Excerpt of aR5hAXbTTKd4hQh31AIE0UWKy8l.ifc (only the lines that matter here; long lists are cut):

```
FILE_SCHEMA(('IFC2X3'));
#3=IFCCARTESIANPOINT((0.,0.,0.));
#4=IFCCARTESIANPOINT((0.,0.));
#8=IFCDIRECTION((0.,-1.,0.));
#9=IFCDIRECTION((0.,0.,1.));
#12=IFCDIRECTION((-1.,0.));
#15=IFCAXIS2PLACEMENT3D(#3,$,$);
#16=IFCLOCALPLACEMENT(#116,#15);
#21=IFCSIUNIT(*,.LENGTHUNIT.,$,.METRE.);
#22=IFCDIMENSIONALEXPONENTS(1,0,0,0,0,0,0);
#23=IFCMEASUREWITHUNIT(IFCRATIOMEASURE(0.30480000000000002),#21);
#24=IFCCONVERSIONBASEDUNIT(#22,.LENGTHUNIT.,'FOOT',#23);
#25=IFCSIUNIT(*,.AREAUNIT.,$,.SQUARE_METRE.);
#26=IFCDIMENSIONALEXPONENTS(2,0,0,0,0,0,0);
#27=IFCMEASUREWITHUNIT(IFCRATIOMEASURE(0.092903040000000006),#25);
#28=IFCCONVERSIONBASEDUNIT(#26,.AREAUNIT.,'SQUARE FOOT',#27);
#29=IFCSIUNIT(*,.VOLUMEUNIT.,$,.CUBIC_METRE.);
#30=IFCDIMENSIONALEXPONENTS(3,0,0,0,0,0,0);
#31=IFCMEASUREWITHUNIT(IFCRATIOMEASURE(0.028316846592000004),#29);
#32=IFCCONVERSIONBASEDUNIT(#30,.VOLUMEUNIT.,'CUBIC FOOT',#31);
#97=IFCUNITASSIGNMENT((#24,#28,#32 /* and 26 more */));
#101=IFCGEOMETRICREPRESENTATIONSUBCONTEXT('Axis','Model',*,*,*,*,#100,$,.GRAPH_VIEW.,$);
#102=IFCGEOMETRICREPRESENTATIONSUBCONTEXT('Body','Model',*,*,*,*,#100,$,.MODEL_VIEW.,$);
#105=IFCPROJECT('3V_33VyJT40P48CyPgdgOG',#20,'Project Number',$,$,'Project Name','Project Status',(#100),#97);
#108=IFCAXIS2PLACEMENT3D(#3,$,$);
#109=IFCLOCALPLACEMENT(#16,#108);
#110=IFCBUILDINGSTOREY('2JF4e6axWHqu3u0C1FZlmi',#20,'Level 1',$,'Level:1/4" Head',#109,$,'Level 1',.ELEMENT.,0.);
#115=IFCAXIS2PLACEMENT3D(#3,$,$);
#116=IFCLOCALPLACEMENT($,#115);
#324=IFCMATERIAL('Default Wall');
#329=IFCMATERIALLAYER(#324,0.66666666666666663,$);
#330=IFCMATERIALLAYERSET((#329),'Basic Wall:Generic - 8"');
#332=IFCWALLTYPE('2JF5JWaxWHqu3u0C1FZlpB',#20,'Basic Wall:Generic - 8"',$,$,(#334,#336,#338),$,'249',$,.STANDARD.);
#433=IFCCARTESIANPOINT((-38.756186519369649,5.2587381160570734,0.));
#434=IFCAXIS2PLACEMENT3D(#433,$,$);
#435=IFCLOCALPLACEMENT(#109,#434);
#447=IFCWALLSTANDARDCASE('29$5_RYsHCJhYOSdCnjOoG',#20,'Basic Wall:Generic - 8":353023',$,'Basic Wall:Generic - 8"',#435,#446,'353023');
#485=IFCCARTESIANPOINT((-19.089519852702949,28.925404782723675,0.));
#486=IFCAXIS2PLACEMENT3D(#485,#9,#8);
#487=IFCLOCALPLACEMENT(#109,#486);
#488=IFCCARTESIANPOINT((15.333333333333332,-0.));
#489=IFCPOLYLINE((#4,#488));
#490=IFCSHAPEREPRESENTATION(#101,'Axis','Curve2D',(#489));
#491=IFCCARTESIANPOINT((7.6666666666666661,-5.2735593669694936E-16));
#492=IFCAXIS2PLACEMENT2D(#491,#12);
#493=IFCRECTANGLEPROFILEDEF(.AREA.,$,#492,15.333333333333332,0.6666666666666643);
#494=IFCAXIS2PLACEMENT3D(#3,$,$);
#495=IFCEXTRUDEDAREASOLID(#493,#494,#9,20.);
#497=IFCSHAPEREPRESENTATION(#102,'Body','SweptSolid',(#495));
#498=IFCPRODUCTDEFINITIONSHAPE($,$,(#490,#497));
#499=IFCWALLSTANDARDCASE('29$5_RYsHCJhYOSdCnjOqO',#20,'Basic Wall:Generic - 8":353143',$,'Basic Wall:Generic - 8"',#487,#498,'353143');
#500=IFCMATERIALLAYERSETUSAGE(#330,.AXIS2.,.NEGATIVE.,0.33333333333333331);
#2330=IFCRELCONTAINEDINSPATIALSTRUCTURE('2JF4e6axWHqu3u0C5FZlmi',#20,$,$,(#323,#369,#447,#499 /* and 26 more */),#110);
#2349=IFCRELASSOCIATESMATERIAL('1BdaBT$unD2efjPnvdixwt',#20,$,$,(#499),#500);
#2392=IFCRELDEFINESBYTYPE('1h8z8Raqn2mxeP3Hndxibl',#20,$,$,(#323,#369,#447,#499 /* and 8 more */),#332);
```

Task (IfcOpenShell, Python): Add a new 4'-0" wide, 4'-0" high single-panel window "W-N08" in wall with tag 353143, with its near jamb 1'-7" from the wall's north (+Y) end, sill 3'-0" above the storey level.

```python
import numpy as np
import ifcopenshell
import ifcopenshell.api.feature
import ifcopenshell.api.geometry
import ifcopenshell.api.root
import ifcopenshell.api.spatial
import ifcopenshell.api.type
import ifcopenshell.geom
import ifcopenshell.util.element
import ifcopenshell.util.placement
import ifcopenshell.util.representation
import ifcopenshell.util.shape
import ifcopenshell.util.unit

model = ifcopenshell.open("aR5hAXbTTKd4hQh31AIE0UWKy8l.ifc")
unit_scale = ifcopenshell.util.unit.calculate_unit_scale(model)
settings = ifcopenshell.geom.settings()


def volume(element):
    """Net volume in cubic metres, openings subtracted."""
    shape = ifcopenshell.geom.create_shape(settings, element)
    return ifcopenshell.util.shape.get_volume(shape.geometry)


wall = model.by_id(499)
storey = ifcopenshell.util.element.get_container(wall, ifc_class="IfcBuildingStorey")
context = ifcopenshell.util.representation.get_context(model, "Model", "Body", "MODEL_VIEW")
before = volume(wall)

width, height, from_end, sill = 1.2192, 1.2192, 0.4826, 0.9144  # metres

# The wall runs along its own X axis, and the end named is its -X end.
wall_shape = ifcopenshell.geom.create_shape(settings, wall)
x, y, z = ifcopenshell.util.shape.get_vertices(wall_shape.geometry).T
start = x.min() + from_end
face, thickness = float(y.min()), float(y.max() - y.min())
wall_matrix = ifcopenshell.util.placement.get_local_placement(wall.ObjectPlacement)
level = ifcopenshell.util.placement.get_local_placement(storey.ObjectPlacement)[2, 3]


def in_wall(x, y):
    """Placement at x, y metres in the wall's axes, at sill height."""
    matrix = wall_matrix.copy()
    matrix[:, 3] = wall_matrix @ np.array([x / unit_scale, y / unit_scale, 0.0, 1.0])
    matrix[2, 3] = level + sill / unit_scale
    return matrix


# Opening: a box that overshoots both wall faces by 50 mm.
opening = ifcopenshell.api.root.create_entity(model, ifc_class="IfcOpeningElement")
box = ifcopenshell.api.geometry.add_wall_representation(
    model, context=context, length=width, height=height, thickness=thickness + 0.1
)
ifcopenshell.api.geometry.assign_representation(model, product=opening, representation=box)
ifcopenshell.api.geometry.edit_object_placement(model, product=opening, matrix=in_wall(start, face - 0.05), is_si=False)
ifcopenshell.api.feature.add_feature(model, feature=opening, element=wall)

window = ifcopenshell.api.root.create_entity(model, ifc_class="IfcWindow", name="W-N08")
window.OverallWidth, window.OverallHeight = width / unit_scale, height / unit_scale
body = ifcopenshell.api.geometry.add_window_representation(
    model,
    context=context,
    overall_width=window.OverallWidth,
    overall_height=window.OverallHeight,
    partition_type="SINGLE_PANEL",
)
ifcopenshell.api.geometry.assign_representation(model, product=window, representation=body)
ifcopenshell.api.spatial.assign_container(model, products=[window], relating_structure=storey)
fills = ifcopenshell.api.feature.add_filling(model, opening=opening, element=window)
fills.OwnerHistory = window.OwnerHistory  # required in IFC2X3

# IFC2X3 keeps the operation on the window style.
style = ifcopenshell.api.root.create_entity(model, ifc_class="IfcWindowStyle", name="W-N08")
style.OperationType, style.ConstructionType = "SINGLE_PANEL", "NOTDEFINED"
style.ParameterTakesPrecedence = style.Sizeable = False
ifcopenshell.api.type.assign_type(model, related_objects=[window], relating_type=style)

# Centre the window in the wall's thickness.
ifcopenshell.api.geometry.edit_object_placement(model, product=window, matrix=in_wall(start, face), is_si=False)
window_shape = ifcopenshell.geom.create_shape(settings, window)
depth = ifcopenshell.util.shape.get_vertices(window_shape.geometry)[:, 1]
offset = face + thickness / 2 - (depth.min() + depth.max()) / 2
ifcopenshell.api.geometry.edit_object_placement(model, product=window, matrix=in_wall(start, offset), is_si=False)

after = volume(wall)

print(f"wall volume {before:.3f} -> {after:.3f} m3")

model.write("aR5hAXbTTKd4hQh31AIE0UWKy8l-out.ifc")
```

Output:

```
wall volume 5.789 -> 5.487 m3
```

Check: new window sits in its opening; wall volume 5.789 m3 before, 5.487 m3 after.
